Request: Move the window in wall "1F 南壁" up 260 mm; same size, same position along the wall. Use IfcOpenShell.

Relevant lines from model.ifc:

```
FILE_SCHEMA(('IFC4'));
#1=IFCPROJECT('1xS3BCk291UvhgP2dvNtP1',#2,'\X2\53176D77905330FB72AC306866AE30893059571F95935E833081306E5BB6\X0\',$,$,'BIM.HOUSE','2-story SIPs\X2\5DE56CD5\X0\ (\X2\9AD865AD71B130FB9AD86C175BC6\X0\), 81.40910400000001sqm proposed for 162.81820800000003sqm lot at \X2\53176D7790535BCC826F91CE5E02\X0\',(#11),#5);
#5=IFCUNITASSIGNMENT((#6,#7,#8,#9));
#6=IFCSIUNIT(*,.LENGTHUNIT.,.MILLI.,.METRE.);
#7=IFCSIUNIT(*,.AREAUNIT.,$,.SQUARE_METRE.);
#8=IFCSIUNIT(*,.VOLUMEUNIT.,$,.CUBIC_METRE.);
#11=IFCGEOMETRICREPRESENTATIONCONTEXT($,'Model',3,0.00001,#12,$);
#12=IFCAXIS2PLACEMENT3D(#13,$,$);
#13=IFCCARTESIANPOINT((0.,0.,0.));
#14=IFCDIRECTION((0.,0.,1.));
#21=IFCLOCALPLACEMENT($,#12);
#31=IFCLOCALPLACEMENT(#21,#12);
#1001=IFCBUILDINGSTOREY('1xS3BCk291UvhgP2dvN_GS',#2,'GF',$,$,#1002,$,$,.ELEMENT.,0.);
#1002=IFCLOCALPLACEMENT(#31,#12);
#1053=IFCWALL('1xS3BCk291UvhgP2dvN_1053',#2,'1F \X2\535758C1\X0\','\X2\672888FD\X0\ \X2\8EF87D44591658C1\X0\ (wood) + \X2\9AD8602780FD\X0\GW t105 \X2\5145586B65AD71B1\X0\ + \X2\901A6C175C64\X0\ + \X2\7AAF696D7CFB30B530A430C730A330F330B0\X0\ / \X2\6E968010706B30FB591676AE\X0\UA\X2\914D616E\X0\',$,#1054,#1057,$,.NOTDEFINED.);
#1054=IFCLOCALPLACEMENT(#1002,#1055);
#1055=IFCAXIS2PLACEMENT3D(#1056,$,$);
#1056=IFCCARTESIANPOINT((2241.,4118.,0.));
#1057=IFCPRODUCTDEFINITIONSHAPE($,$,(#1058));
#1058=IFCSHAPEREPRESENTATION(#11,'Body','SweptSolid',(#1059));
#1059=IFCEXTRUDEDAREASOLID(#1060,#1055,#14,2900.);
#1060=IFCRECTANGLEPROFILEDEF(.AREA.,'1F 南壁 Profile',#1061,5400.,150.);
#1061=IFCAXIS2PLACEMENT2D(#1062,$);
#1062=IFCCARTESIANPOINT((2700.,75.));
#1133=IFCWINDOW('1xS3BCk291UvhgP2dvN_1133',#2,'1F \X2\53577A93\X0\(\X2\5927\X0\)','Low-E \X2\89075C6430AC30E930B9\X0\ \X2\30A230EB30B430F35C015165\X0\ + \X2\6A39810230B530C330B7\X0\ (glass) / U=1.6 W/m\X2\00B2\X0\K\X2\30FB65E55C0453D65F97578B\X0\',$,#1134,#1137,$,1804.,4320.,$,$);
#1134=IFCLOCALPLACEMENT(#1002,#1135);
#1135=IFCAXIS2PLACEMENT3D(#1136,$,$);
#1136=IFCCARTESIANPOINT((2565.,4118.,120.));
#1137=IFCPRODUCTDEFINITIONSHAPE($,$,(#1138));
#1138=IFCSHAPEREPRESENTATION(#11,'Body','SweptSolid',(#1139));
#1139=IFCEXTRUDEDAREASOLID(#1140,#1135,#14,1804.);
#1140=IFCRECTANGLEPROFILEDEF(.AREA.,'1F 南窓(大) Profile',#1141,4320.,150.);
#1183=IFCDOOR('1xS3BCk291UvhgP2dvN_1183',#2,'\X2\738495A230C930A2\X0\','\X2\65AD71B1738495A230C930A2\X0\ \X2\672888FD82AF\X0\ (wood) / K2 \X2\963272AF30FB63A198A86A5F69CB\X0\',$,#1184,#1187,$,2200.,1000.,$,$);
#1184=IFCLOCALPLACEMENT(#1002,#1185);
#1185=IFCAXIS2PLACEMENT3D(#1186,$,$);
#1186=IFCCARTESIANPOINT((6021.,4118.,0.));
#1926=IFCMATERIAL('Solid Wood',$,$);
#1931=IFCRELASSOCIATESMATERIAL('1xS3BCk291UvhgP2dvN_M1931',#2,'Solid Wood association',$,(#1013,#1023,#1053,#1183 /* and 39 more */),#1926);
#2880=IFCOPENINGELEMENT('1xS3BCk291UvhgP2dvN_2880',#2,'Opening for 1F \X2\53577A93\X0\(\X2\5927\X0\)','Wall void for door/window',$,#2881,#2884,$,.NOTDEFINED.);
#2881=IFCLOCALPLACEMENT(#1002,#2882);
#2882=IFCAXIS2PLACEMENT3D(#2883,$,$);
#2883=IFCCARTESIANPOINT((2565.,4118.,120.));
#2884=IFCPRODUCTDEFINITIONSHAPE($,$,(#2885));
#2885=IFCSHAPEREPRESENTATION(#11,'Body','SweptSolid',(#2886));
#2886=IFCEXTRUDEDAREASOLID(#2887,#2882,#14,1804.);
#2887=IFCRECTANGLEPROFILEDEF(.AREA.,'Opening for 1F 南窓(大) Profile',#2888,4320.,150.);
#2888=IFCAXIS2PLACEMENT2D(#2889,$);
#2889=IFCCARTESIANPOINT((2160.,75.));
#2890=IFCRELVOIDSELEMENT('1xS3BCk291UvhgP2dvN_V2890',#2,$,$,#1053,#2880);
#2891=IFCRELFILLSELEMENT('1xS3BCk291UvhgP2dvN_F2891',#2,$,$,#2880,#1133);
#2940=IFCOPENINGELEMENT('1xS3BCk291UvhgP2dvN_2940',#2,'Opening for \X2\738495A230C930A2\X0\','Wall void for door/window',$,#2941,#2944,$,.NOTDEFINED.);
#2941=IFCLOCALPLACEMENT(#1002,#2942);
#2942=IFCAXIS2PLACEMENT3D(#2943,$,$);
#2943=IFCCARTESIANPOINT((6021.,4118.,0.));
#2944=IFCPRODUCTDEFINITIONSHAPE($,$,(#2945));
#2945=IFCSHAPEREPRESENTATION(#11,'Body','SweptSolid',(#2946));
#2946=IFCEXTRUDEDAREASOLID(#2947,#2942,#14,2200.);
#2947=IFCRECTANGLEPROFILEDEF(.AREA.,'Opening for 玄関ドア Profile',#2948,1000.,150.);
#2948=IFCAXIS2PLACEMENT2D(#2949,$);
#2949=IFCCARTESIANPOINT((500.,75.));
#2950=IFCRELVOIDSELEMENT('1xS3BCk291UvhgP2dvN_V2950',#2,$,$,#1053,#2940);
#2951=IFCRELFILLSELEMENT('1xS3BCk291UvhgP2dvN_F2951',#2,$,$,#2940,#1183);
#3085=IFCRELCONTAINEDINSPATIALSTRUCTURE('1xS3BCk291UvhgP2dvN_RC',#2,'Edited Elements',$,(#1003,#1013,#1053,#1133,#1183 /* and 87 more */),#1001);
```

```python
import numpy as np
import ifcopenshell
import ifcopenshell.api.geometry
import ifcopenshell.util.placement
import ifcopenshell.util.unit

model = ifcopenshell.open("model.ifc")
unit_scale = ifcopenshell.util.unit.calculate_unit_scale(model)

window = model.by_guid("1xS3BCk291UvhgP2dvN_1133")
opening = window.FillsVoids[0].RelatingOpeningElement
dz = 0.26 / unit_scale

shift = np.array([0.0, 0.0, dz])
# The window is not placed relative to its opening, so move both.
for product in (opening, window):
    matrix = ifcopenshell.util.placement.get_local_placement(product.ObjectPlacement)
    matrix[:3, 3] += shift
    ifcopenshell.api.geometry.edit_object_placement(model, product=product, matrix=matrix, is_si=False)

print(f"moved by {dz * unit_scale:+.3f} m")

model.write("model_rev.ifc")
```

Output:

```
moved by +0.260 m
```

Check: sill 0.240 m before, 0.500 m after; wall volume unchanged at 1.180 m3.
